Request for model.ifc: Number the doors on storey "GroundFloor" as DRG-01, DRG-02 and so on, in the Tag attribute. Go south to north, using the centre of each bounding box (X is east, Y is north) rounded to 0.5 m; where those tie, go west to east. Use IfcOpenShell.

First a look at what the model holds.

```python
import ifcopenshell
import ifcopenshell.util.element
import ifcopenshell.util.placement

model = ifcopenshell.open("model.ifc")
print(model.schema)
storey = next(s for s in model.by_type("IfcBuildingStorey") if s.Name == "GroundFloor")
doors = [e for e in ifcopenshell.util.element.get_decomposition(storey) if e.is_a("IfcDoor")]
for e in sorted(doors, key=lambda e: e.id()):
    origin = ifcopenshell.util.placement.get_local_placement(e.ObjectPlacement)[:3, 3]
    print(e.id(), e.Tag, e.Name, origin.round(2) + 0.0, sep=" | ")
```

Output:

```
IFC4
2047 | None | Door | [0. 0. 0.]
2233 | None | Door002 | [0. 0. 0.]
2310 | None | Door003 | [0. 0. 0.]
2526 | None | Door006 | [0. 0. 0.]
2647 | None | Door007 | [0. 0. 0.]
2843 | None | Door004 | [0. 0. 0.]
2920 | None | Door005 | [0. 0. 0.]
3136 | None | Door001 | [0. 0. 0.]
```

```python
import ifcopenshell
import ifcopenshell.geom
import ifcopenshell.util.element
import ifcopenshell.util.shape

model = ifcopenshell.open("model.ifc")
settings = ifcopenshell.geom.settings()
settings.set("use-world-coords", True)


def centre(element):
    shape = ifcopenshell.geom.create_shape(settings, element)
    return ifcopenshell.util.shape.get_bbox_centroid(shape.geometry)


storey = next(s for s in model.by_type("IfcBuildingStorey") if s.Name == "GroundFloor")
doors = [e for e in ifcopenshell.util.element.get_decomposition(storey) if e.is_a("IfcDoor")]

# Insertion points can sit at a corner or the storey origin, so sort by the geometry (in metres).
centres = {e: centre(e) for e in doors}
doors.sort(key=lambda e: (round(centres[e][1] / 0.5), centres[e][0]))

for i, e in enumerate(doors, start=1):
    number = f"DRG-{i:02d}"
    e.Tag = number
    print(e.id(), number)

model.write("model_v2.ifc")
```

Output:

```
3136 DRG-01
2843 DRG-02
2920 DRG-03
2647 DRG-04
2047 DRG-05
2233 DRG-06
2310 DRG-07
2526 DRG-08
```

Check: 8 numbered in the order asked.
